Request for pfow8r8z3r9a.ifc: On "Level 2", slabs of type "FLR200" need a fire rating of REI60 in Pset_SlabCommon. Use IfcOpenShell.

First a look at what the model holds.

```python
import ifcopenshell
import ifcopenshell.util.element

model = ifcopenshell.open("pfow8r8z3r9a.ifc")
print(model.schema)
storey = next(s for s in model.by_type("IfcBuildingStorey") if s.Name == "Level 2")
slabs = [e for e in ifcopenshell.util.element.get_decomposition(storey) if e.is_a("IfcSlab")]
seen = {}
for e in slabs:
    element_type = ifcopenshell.util.element.get_type(e)
    key = (element_type.Name if element_type != e and element_type else None, ifcopenshell.util.element.get_pset(e, "Pset_SlabCommon", "FireRating"))
    seen[key] = seen.get(key, 0) + 1
for (name, value), count in sorted(seen.items(), key=str):
    print(count, "x", name, "|", value)
```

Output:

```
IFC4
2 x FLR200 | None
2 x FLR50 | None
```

```python
import ifcopenshell
import ifcopenshell.api.pset
import ifcopenshell.util.element

model = ifcopenshell.open("pfow8r8z3r9a.ifc")

storey = next(s for s in model.by_type("IfcBuildingStorey") if s.Name == "Level 2")
slabs = [e for e in ifcopenshell.util.element.get_decomposition(storey) if e.is_a("IfcSlab")]

count = 0
for e in slabs:
    element_type = ifcopenshell.util.element.get_type(e)
    if element_type in (None, e) or element_type.Name != "FLR200":
        continue
    # add_pset returns the element's existing set when there is one.
    pset = ifcopenshell.api.pset.add_pset(model, product=e, name="Pset_SlabCommon")
    ifcopenshell.api.pset.edit_pset(model, pset=pset, properties={"FireRating": "REI60"})
    count += 1

print(count, "slabs updated")

model.write("pfow8r8z3r9a_v2.ifc")
```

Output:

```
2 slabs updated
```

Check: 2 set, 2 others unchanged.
